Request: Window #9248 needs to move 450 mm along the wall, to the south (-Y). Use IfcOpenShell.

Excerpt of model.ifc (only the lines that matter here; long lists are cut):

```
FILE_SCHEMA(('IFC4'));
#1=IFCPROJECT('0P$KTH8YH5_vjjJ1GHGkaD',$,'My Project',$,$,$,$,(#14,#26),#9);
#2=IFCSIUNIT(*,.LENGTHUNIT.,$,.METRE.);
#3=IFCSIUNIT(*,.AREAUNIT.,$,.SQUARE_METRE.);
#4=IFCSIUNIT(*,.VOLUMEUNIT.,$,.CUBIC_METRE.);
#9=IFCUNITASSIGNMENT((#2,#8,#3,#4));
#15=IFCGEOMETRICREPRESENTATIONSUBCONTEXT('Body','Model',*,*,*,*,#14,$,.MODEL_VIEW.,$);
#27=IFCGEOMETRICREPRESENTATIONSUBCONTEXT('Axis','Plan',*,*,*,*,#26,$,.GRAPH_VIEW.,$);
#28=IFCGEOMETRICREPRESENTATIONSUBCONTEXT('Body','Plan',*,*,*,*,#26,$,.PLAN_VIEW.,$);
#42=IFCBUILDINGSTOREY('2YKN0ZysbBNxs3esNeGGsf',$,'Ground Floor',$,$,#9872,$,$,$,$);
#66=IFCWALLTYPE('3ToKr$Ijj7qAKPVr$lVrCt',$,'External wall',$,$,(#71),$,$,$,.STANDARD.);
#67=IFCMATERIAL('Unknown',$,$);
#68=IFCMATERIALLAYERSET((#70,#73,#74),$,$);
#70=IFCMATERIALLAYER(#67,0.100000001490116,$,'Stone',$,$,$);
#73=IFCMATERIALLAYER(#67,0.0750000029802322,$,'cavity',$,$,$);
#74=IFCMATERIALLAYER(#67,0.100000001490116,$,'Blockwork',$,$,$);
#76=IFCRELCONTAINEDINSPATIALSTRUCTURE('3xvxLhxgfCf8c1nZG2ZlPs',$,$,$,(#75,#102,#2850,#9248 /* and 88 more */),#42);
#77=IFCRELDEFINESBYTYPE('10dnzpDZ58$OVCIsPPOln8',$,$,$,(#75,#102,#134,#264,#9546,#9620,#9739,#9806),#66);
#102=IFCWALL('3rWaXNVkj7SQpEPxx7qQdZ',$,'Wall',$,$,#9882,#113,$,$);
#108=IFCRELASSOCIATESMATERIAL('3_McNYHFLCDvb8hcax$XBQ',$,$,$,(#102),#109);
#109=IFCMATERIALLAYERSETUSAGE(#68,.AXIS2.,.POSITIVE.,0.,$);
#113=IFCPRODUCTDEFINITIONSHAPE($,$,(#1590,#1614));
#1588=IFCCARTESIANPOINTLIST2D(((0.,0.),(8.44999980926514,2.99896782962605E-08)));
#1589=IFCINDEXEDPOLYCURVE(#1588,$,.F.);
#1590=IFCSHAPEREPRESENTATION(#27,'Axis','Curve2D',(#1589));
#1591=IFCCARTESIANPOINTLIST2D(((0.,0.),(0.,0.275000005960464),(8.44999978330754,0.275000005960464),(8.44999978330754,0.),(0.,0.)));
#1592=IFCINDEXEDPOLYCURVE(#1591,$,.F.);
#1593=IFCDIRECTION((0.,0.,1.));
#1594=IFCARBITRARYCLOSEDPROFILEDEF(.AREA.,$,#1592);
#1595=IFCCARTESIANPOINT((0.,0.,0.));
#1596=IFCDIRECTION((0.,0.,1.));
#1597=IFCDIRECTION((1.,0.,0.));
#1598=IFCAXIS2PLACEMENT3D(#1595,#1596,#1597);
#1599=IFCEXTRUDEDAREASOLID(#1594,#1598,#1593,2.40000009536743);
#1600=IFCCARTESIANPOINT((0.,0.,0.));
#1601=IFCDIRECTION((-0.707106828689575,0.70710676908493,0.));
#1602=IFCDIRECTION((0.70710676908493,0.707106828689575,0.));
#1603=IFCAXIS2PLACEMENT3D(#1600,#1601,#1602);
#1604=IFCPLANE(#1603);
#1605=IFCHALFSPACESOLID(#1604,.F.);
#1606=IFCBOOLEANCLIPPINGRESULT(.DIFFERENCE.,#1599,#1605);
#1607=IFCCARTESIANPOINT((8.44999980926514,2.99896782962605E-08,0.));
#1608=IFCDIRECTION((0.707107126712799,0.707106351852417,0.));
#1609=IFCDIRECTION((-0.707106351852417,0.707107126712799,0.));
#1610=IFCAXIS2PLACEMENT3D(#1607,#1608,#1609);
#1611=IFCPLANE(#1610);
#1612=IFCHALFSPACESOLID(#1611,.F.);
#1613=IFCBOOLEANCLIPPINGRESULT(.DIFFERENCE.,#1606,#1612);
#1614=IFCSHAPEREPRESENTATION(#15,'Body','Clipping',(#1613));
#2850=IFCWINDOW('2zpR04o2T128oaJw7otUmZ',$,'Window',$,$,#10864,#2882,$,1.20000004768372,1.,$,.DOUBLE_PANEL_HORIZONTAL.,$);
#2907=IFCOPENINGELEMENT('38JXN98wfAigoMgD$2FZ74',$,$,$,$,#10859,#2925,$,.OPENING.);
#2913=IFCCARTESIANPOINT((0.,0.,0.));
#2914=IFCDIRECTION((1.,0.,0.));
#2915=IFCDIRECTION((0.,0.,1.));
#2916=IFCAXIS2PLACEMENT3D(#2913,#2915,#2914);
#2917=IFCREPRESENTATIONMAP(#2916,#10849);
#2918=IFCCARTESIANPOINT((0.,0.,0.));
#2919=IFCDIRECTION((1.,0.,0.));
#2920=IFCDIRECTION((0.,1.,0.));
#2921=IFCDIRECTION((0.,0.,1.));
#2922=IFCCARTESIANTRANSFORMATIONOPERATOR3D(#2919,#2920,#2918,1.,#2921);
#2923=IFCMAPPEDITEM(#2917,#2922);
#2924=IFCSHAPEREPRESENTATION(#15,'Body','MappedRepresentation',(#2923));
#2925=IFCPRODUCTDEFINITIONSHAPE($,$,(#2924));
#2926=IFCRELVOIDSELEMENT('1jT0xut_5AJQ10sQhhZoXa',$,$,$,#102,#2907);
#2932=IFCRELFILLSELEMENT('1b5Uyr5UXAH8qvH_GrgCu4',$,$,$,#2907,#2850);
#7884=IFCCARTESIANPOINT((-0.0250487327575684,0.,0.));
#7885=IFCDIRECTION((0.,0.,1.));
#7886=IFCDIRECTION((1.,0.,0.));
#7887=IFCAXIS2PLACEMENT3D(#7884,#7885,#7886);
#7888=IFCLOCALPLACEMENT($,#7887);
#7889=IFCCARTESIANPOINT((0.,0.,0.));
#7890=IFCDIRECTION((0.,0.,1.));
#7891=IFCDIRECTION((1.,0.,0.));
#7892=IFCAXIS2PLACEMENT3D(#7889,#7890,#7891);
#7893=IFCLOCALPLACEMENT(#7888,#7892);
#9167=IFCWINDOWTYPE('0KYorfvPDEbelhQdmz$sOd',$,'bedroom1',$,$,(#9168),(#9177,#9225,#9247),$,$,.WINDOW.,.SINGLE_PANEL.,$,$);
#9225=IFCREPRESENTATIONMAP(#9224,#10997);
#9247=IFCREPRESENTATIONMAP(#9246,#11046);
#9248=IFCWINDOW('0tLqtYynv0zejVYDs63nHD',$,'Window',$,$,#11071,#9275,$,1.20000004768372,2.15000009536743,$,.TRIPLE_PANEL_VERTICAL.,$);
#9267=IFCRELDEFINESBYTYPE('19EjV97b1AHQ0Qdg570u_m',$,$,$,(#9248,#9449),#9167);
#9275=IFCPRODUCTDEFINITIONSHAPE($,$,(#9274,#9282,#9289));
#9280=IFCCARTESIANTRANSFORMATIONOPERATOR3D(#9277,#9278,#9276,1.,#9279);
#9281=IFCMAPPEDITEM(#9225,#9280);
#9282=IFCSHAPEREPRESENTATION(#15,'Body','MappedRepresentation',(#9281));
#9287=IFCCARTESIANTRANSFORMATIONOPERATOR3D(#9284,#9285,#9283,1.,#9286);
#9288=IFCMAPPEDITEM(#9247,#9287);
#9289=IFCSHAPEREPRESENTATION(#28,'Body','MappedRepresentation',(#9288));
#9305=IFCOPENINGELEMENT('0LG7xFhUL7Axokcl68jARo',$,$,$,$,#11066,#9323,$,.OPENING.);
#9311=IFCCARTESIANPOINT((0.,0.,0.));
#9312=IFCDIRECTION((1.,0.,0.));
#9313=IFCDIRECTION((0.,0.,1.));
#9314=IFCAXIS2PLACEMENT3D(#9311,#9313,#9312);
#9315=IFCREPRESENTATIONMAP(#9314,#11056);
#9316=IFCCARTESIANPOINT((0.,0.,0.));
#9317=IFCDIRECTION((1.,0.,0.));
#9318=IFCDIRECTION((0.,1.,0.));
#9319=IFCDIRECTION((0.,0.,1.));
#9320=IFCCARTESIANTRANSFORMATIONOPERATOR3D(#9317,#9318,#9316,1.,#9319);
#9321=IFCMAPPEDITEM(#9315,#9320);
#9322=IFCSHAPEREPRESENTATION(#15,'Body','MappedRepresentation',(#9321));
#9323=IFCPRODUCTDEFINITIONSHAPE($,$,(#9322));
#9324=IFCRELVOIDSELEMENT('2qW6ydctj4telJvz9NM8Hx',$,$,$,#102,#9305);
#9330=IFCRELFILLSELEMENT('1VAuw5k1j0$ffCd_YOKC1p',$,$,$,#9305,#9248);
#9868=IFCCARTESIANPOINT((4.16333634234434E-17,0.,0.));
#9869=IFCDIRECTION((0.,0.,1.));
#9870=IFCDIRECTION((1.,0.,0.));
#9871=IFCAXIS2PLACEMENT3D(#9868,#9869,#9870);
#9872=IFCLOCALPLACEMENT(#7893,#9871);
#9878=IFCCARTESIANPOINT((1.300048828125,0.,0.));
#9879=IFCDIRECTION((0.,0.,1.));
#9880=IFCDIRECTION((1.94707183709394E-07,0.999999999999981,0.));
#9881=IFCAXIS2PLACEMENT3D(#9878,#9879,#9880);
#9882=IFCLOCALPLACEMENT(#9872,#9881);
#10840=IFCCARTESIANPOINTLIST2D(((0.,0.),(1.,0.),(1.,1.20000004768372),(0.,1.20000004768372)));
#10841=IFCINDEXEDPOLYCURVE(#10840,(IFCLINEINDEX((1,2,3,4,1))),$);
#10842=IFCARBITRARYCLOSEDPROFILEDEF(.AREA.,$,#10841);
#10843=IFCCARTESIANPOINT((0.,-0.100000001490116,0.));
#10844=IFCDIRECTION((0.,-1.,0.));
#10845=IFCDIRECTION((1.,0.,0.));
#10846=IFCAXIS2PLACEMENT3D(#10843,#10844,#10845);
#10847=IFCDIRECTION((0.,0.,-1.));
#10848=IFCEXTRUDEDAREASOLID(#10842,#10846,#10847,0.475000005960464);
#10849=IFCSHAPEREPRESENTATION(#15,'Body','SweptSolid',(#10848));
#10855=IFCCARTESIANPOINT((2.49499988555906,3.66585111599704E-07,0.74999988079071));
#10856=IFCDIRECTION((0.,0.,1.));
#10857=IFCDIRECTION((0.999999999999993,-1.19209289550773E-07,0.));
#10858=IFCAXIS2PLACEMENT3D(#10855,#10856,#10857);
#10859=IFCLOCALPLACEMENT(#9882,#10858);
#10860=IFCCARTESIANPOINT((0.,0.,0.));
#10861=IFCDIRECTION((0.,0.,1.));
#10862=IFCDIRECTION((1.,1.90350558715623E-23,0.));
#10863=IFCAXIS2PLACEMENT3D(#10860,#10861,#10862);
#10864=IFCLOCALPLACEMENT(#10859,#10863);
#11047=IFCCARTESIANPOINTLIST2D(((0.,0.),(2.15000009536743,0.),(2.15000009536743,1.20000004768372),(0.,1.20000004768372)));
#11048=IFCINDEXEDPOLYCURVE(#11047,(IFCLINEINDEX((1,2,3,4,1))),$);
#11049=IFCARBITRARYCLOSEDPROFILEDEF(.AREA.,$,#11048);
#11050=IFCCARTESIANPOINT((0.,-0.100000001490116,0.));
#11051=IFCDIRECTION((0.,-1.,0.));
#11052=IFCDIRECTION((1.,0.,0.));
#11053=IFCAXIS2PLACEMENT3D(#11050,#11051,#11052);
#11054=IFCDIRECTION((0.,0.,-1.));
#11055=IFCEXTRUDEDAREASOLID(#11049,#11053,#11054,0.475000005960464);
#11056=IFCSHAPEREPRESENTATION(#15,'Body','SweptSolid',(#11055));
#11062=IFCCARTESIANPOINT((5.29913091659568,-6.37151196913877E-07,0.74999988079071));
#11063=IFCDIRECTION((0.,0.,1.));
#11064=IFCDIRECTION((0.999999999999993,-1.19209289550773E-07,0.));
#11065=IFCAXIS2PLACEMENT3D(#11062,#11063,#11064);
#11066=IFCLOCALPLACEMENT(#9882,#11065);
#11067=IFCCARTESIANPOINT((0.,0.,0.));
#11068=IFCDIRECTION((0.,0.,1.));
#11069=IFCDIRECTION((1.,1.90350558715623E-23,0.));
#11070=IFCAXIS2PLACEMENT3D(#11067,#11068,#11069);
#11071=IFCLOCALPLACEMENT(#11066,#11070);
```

```python
import ifcopenshell
import ifcopenshell.api.geometry
import ifcopenshell.util.placement

model = ifcopenshell.open("model.ifc")

window = model.by_guid("0tLqtYynv0zejVYDs63nHD")
opening = window.FillsVoids[0].RelatingOpeningElement
wall = opening.VoidsElements[0].RelatingBuildingElement

wall_matrix = ifcopenshell.util.placement.get_local_placement(wall.ObjectPlacement)
shift = wall_matrix[:3, 0] * -0.45
before = ifcopenshell.util.placement.get_local_placement(window.ObjectPlacement)[:3, 3].copy()

# The window is placed relative to its opening, so it follows when the opening moves.
matrix = ifcopenshell.util.placement.get_local_placement(opening.ObjectPlacement)
matrix[:3, 3] += shift
ifcopenshell.api.geometry.edit_object_placement(
    model, product=opening, matrix=matrix, is_si=False, should_transform_children=True
)

after = ifcopenshell.util.placement.get_local_placement(window.ObjectPlacement)[:3, 3]
print("window moved by", (after - before).round(3) + 0.0)

model.write("model_v2.ifc")
```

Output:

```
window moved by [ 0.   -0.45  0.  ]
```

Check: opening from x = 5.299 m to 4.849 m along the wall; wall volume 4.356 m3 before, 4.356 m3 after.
